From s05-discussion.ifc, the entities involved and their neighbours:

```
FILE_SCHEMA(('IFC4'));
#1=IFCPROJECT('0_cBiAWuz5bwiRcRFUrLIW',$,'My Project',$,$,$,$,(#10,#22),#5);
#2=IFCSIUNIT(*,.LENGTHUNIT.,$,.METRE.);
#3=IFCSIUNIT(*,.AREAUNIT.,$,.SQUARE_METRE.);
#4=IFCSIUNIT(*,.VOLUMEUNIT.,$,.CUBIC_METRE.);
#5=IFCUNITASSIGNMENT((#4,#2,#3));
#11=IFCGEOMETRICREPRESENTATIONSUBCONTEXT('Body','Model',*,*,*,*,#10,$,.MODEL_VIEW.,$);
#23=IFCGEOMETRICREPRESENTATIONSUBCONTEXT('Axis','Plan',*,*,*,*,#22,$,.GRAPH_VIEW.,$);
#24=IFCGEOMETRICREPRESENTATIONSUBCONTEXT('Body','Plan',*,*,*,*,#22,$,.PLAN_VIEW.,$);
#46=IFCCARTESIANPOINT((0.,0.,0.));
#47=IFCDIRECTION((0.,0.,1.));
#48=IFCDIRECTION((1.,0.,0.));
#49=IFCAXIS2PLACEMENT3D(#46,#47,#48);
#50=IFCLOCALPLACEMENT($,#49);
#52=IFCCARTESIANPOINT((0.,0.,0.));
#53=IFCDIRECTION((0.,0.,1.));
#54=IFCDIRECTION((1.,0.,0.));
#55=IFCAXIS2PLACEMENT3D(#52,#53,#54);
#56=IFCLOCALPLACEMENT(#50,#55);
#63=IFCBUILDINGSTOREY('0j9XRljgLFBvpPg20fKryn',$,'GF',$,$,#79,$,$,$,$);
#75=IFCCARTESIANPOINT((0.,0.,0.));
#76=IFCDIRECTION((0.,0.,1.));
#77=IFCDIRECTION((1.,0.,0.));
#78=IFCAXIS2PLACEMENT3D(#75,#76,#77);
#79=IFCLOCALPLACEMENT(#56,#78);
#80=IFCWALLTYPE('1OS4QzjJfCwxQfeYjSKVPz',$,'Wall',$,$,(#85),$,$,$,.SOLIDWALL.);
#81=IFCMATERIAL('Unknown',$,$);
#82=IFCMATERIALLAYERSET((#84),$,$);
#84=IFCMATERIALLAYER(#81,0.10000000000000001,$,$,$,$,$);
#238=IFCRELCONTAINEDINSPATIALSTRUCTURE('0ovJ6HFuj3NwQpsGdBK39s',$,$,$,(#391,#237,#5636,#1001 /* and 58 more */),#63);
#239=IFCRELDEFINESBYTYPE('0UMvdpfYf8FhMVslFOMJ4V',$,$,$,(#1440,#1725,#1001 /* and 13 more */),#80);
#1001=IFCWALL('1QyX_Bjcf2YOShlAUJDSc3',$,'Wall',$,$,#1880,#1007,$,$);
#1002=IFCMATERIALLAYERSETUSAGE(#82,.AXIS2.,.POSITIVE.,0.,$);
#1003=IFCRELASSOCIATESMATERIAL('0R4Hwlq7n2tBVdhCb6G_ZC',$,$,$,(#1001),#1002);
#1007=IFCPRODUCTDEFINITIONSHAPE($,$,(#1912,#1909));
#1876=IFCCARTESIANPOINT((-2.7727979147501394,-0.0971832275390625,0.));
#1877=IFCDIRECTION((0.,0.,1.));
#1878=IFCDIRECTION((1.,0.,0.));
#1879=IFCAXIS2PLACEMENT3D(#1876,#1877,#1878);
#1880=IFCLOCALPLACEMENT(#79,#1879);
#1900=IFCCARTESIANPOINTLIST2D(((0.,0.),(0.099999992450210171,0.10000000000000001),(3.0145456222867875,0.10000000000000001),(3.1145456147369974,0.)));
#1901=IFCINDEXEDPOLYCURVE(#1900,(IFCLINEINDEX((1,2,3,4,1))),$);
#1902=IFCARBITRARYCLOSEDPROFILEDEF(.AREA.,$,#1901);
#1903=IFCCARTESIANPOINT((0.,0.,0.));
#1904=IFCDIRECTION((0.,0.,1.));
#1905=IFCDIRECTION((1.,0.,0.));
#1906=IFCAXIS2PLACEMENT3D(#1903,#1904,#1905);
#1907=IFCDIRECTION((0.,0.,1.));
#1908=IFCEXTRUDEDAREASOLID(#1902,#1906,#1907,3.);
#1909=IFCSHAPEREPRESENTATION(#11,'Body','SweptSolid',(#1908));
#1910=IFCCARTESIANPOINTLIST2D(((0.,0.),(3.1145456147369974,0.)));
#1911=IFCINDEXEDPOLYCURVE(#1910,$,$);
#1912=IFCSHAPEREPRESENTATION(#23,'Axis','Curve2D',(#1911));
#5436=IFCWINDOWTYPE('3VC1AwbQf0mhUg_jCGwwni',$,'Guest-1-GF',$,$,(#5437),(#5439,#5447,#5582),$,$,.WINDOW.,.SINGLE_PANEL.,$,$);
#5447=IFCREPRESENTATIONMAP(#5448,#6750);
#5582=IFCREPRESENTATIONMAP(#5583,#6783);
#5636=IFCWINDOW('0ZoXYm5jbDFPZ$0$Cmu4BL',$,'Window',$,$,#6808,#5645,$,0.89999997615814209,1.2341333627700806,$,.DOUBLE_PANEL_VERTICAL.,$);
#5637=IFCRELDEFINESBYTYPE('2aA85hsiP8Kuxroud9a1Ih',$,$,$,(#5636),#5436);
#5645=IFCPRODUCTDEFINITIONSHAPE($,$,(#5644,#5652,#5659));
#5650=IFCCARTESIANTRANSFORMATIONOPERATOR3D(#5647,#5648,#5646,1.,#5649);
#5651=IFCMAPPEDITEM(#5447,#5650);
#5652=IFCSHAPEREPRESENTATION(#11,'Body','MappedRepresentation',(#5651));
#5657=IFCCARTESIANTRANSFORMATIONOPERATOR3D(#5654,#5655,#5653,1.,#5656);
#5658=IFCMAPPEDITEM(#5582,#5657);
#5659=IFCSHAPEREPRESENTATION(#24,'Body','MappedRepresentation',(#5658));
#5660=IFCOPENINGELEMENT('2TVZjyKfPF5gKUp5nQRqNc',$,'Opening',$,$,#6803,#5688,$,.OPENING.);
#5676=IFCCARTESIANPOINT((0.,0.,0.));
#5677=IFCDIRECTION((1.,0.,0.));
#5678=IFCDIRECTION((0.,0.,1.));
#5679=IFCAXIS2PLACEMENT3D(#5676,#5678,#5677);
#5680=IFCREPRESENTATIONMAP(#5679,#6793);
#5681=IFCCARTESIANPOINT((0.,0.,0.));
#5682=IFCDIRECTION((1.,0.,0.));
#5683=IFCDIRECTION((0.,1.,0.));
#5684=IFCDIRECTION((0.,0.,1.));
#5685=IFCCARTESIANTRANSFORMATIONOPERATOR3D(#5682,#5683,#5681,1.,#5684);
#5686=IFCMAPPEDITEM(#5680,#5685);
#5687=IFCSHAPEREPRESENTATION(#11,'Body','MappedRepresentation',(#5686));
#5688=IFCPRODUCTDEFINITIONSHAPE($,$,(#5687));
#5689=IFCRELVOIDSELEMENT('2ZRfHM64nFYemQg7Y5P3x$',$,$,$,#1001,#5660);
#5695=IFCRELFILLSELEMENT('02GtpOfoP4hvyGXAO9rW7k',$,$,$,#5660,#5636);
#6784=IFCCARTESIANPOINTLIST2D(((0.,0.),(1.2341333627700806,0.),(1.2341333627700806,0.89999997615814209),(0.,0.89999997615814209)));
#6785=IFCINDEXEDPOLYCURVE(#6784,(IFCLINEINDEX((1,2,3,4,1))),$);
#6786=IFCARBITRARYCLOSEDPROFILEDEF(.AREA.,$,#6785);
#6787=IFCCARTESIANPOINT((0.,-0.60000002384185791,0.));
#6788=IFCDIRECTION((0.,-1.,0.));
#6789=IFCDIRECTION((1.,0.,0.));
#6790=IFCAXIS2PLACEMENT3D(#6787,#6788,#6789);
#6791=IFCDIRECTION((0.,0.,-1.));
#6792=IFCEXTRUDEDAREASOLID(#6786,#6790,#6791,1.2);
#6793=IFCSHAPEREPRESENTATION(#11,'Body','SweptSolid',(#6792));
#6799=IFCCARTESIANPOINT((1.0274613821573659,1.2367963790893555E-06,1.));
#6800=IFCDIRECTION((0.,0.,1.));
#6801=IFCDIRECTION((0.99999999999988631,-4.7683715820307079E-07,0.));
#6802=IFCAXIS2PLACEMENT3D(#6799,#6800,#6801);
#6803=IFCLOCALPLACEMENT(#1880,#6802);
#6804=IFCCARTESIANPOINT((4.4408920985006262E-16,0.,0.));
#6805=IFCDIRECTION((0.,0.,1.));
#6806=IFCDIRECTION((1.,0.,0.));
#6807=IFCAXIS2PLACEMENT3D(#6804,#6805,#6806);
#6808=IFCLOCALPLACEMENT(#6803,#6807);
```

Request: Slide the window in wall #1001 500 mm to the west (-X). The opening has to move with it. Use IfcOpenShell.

```python
import ifcopenshell
import ifcopenshell.api.geometry
import ifcopenshell.util.placement
import ifcopenshell.util.unit

model = ifcopenshell.open("s05-discussion.ifc")
unit_scale = ifcopenshell.util.unit.calculate_unit_scale(model)

window = model.by_guid("0ZoXYm5jbDFPZ$0$Cmu4BL")
opening = window.FillsVoids[0].RelatingOpeningElement
wall = opening.VoidsElements[0].RelatingBuildingElement

wall_matrix = ifcopenshell.util.placement.get_local_placement(wall.ObjectPlacement)
shift = wall_matrix[:3, 0] * -0.5 / unit_scale
before = ifcopenshell.util.placement.get_local_placement(window.ObjectPlacement)[:3, 3].copy()

# The window is placed relative to its opening, so it follows when the opening moves.
matrix = ifcopenshell.util.placement.get_local_placement(opening.ObjectPlacement)
matrix[:3, 3] += shift
ifcopenshell.api.geometry.edit_object_placement(
    model, product=opening, matrix=matrix, is_si=False, should_transform_children=True
)

after = ifcopenshell.util.placement.get_local_placement(window.ObjectPlacement)[:3, 3]
print("window moved by", (after - before).round(3) + 0.0)

model.write("s05-discussion_updated.ifc")
```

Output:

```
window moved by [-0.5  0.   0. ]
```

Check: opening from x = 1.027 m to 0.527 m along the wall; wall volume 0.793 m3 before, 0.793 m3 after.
